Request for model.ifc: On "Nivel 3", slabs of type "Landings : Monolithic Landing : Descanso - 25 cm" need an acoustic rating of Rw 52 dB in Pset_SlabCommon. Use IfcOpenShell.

First a look at what the model holds.

```python
import ifcopenshell
import ifcopenshell.util.element

model = ifcopenshell.open("model.ifc")
print(model.schema)
storey = next(s for s in model.by_type("IfcBuildingStorey") if s.Name == "Nivel 3")
slabs = [e for e in ifcopenshell.util.element.get_decomposition(storey) if e.is_a("IfcSlab")]
seen = {}
for e in slabs:
    element_type = ifcopenshell.util.element.get_type(e)
    key = (element_type.Name if element_type != e and element_type else None, ifcopenshell.util.element.get_pset(e, "Pset_SlabCommon", "AcousticRating"))
    seen[key] = seen.get(key, 0) + 1
for (name, value), count in sorted(seen.items(), key=str):
    print(count, "x", name, "|", value)
```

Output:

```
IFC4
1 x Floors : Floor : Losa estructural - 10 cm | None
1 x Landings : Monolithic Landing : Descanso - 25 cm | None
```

```python
import ifcopenshell
import ifcopenshell.api.pset
import ifcopenshell.util.element

model = ifcopenshell.open("model.ifc")

storey = next(s for s in model.by_type("IfcBuildingStorey") if s.Name == "Nivel 3")
slabs = [e for e in ifcopenshell.util.element.get_decomposition(storey) if e.is_a("IfcSlab")]

count = 0
for e in slabs:
    element_type = ifcopenshell.util.element.get_type(e)
    if element_type in (None, e) or element_type.Name != "Landings : Monolithic Landing : Descanso - 25 cm":
        continue
    # add_pset returns the element's existing set when there is one.
    pset = ifcopenshell.api.pset.add_pset(model, product=e, name="Pset_SlabCommon")
    ifcopenshell.api.pset.edit_pset(model, pset=pset, properties={"AcousticRating": "Rw 52 dB"})
    count += 1

print(count, "slabs updated")

model.write("model_rev.ifc")
```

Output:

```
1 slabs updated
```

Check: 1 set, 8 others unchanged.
